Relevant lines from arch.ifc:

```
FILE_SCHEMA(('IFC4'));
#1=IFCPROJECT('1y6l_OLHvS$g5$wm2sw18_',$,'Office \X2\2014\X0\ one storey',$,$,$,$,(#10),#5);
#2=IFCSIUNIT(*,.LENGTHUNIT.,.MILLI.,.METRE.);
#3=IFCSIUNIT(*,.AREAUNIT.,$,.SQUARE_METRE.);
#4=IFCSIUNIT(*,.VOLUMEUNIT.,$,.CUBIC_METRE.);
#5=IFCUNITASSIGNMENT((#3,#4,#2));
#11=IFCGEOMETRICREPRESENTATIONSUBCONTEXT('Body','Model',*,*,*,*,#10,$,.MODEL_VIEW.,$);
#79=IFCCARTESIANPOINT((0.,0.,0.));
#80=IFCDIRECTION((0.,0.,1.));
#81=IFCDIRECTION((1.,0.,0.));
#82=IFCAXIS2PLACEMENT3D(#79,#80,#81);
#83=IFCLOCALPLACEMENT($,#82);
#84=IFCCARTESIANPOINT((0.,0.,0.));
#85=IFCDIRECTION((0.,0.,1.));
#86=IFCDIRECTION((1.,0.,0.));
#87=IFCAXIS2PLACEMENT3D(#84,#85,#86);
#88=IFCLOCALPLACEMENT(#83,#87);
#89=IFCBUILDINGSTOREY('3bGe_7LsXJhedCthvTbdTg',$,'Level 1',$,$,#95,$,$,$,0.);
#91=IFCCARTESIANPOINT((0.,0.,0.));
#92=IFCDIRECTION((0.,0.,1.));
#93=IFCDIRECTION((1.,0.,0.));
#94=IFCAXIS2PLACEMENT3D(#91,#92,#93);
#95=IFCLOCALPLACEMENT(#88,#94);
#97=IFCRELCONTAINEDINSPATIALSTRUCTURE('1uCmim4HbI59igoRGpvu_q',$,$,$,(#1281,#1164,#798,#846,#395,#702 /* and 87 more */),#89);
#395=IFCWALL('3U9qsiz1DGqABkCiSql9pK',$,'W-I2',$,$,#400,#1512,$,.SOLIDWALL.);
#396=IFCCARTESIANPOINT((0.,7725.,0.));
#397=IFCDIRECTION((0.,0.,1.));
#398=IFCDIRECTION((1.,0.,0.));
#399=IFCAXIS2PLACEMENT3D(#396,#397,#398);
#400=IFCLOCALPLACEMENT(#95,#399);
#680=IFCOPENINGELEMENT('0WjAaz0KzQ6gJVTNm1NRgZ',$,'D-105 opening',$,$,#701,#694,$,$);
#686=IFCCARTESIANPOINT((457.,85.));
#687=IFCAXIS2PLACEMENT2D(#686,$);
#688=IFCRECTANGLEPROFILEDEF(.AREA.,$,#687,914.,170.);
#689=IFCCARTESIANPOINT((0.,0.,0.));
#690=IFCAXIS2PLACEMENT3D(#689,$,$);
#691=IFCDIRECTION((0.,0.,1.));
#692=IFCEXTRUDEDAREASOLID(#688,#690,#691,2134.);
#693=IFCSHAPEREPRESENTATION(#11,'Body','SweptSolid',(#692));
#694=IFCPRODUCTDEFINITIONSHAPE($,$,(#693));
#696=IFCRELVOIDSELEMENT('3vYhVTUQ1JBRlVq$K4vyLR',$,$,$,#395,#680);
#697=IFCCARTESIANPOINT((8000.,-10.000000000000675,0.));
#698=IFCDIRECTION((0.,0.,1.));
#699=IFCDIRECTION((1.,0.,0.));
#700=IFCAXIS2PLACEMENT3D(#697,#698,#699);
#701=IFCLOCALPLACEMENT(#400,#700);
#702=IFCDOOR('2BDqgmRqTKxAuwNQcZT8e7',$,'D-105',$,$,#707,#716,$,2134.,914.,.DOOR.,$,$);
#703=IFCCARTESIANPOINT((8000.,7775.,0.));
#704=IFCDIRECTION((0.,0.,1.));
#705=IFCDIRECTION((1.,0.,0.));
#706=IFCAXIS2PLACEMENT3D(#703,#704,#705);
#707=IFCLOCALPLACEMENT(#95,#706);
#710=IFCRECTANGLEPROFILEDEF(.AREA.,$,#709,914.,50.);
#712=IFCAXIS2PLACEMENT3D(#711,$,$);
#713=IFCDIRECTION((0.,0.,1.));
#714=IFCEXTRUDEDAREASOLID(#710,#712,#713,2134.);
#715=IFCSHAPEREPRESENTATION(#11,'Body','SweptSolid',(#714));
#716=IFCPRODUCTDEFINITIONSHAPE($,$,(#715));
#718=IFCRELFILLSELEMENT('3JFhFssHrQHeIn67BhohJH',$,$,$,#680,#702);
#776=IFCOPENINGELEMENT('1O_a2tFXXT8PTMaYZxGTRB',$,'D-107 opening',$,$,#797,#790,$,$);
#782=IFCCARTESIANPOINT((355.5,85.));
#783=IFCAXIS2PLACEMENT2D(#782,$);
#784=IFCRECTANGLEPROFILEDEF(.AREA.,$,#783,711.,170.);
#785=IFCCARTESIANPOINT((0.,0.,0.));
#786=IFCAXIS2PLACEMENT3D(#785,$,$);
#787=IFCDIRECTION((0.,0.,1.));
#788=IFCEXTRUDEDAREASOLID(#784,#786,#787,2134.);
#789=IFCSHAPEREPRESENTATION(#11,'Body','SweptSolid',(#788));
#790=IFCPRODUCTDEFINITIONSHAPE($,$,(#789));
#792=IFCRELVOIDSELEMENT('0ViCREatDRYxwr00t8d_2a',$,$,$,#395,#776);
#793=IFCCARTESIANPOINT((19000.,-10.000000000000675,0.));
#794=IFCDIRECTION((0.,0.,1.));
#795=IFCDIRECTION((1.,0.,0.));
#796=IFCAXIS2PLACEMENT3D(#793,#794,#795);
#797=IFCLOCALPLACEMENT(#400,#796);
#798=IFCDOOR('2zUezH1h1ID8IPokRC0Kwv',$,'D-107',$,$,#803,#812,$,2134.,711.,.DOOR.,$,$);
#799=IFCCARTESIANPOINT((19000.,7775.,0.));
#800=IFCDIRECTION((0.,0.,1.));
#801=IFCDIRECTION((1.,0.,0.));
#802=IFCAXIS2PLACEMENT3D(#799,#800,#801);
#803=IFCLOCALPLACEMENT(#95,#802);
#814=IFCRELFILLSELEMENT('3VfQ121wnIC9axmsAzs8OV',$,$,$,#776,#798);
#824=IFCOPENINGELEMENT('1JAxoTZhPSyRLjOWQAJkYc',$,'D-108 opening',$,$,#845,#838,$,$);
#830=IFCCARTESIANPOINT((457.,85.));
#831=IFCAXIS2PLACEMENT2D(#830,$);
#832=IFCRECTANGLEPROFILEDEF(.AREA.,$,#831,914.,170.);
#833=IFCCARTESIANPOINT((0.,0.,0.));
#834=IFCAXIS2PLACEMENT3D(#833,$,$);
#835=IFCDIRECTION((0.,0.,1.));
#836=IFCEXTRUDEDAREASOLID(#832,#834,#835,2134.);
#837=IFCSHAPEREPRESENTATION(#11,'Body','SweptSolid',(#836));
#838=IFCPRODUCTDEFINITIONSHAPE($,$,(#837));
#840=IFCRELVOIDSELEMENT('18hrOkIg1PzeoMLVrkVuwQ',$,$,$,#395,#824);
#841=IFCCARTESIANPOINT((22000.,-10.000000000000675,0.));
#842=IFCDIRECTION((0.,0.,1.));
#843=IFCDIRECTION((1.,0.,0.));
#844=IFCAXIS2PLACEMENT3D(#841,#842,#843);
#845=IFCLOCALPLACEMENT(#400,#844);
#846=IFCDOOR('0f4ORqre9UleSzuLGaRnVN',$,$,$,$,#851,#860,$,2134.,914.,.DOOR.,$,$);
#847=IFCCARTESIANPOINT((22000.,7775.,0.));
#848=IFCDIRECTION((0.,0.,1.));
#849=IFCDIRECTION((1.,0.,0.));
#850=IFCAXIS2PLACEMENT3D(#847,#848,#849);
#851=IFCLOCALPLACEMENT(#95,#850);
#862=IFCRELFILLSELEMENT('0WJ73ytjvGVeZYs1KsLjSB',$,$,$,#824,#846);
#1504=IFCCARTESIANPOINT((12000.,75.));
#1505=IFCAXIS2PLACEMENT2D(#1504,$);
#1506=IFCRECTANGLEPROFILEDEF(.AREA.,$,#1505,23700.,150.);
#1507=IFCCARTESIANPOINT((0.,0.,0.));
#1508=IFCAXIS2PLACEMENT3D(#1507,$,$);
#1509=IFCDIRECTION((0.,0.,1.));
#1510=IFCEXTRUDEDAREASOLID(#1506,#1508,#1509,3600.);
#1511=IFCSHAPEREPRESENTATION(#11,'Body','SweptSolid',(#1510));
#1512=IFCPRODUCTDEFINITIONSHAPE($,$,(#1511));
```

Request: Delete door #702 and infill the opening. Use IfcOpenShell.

```python
import ifcopenshell
import ifcopenshell.api.feature
import ifcopenshell.api.root
import ifcopenshell.geom
import ifcopenshell.util.shape

model = ifcopenshell.open("arch.ifc")
settings = ifcopenshell.geom.settings()


def volume(element):
    """Net volume in cubic metres, openings subtracted."""
    shape = ifcopenshell.geom.create_shape(settings, element)
    return ifcopenshell.util.shape.get_volume(shape.geometry)


door = model.by_guid("2BDqgmRqTKxAuwNQcZT8e7")
opening = door.FillsVoids[0].RelatingOpeningElement
wall = opening.VoidsElements[0].RelatingBuildingElement
before = volume(wall)

ifcopenshell.api.root.remove_product(model, product=door)
ifcopenshell.api.feature.remove_feature(model, feature=opening)

after = volume(wall)

print(f"wall volume {before:.3f} -> {after:.3f} m3")

model.write("arch_v2.ifc")
```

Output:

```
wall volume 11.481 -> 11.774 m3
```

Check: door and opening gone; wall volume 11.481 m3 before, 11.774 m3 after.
